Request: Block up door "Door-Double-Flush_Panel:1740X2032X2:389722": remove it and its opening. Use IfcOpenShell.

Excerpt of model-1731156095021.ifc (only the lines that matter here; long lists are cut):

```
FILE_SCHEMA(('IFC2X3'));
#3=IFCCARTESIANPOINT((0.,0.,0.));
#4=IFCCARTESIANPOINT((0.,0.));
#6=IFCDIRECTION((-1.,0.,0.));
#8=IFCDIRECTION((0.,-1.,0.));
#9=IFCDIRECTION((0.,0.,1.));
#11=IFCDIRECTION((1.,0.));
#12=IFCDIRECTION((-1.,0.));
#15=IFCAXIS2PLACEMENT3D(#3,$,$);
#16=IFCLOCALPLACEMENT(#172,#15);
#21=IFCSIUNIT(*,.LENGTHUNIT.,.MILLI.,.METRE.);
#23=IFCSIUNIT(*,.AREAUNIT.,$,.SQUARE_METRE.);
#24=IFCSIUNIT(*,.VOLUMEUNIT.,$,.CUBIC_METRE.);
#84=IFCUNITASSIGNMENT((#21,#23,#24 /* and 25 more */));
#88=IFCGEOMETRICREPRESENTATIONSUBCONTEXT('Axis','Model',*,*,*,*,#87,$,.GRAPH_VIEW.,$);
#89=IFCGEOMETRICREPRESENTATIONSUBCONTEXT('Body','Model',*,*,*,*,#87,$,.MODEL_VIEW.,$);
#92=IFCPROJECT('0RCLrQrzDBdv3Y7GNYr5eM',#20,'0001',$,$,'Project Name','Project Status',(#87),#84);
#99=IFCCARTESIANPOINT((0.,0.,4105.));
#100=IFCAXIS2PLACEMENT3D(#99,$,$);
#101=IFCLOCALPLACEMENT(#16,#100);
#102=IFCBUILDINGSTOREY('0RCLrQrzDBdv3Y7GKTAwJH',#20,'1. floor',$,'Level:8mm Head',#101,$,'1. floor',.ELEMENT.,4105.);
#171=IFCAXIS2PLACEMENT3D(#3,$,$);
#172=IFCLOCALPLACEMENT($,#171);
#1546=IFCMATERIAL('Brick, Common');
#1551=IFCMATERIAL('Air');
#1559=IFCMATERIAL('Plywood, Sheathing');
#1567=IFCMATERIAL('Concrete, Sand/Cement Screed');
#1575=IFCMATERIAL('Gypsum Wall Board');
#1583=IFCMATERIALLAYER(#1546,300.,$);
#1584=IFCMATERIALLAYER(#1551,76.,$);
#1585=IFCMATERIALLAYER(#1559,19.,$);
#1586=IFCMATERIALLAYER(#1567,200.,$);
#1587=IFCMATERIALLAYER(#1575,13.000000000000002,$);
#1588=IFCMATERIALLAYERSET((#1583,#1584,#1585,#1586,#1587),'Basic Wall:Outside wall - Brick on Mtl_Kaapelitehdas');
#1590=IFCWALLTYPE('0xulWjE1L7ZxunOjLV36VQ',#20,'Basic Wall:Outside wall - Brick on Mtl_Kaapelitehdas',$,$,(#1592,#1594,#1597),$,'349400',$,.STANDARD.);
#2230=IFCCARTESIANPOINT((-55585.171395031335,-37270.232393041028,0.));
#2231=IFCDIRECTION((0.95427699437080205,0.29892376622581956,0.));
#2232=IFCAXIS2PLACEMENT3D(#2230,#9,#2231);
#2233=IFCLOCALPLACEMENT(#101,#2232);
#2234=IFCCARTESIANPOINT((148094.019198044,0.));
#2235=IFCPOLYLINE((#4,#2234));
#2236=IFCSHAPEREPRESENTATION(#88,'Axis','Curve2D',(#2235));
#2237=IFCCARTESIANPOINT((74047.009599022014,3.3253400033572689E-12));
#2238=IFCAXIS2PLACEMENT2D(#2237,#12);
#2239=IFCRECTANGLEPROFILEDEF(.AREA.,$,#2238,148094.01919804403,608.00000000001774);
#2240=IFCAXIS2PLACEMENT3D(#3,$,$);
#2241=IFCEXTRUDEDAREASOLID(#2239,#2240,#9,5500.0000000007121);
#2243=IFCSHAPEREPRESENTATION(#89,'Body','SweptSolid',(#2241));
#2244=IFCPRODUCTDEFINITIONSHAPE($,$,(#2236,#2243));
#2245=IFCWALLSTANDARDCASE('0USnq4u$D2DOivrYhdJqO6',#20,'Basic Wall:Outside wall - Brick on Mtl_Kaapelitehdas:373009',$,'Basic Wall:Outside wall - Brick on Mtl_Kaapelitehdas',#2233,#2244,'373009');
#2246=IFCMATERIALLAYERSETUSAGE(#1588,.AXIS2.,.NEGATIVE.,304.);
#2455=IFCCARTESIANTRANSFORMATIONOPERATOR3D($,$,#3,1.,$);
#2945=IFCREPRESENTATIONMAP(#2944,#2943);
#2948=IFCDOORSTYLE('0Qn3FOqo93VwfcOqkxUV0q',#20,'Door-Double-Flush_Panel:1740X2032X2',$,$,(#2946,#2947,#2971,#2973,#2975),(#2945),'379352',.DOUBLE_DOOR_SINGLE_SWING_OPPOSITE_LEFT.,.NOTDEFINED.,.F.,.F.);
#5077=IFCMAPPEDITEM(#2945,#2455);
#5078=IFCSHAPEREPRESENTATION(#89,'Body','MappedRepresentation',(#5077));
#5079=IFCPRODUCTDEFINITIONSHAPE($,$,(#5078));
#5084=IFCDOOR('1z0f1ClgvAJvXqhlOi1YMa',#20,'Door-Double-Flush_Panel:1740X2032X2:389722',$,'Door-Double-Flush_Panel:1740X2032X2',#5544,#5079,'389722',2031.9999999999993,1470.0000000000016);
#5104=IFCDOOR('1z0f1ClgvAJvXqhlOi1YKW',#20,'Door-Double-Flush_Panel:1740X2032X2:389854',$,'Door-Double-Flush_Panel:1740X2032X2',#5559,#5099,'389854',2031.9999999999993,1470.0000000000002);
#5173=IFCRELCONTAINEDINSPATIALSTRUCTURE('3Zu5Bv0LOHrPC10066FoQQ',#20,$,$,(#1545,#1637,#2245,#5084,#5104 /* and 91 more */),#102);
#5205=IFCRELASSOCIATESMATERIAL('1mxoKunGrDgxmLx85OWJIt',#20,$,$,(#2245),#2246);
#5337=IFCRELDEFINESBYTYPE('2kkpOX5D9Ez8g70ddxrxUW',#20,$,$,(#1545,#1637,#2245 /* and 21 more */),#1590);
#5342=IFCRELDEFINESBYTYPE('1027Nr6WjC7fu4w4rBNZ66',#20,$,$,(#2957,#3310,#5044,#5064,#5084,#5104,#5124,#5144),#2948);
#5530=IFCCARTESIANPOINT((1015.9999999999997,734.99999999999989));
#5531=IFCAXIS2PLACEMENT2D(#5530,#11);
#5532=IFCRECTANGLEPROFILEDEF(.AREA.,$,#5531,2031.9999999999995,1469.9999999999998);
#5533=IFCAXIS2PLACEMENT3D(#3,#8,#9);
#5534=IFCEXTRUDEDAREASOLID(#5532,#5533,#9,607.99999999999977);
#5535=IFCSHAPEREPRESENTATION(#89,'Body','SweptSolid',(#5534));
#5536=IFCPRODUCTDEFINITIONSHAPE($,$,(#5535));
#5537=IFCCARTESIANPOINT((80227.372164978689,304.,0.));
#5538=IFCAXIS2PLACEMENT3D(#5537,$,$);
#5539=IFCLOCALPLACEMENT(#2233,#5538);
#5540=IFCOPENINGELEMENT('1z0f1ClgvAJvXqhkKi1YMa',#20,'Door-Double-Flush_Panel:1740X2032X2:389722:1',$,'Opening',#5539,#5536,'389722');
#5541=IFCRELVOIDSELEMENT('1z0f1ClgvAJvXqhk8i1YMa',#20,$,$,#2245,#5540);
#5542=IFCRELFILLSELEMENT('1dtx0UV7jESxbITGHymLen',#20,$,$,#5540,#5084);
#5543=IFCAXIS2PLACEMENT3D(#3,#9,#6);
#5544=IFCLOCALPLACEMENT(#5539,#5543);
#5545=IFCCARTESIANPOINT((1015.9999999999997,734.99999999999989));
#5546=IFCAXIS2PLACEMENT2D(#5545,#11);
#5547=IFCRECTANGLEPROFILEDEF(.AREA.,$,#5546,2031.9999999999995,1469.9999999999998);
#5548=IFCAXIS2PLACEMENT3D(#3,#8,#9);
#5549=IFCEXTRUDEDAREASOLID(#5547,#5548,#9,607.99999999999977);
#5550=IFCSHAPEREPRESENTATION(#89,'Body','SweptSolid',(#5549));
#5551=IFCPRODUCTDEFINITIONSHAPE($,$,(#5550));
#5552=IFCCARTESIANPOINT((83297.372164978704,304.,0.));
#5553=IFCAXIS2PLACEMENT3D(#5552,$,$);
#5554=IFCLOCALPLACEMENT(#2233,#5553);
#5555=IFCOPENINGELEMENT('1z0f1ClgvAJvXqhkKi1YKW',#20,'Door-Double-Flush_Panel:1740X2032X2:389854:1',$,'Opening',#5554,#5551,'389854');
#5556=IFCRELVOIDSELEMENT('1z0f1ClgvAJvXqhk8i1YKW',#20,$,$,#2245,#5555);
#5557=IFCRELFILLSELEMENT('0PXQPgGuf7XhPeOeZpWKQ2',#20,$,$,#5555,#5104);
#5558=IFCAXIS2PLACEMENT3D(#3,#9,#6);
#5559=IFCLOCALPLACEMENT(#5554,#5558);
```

```python
import ifcopenshell
import ifcopenshell.api.feature
import ifcopenshell.api.root
import ifcopenshell.geom
import ifcopenshell.util.shape

model = ifcopenshell.open("model-1731156095021.ifc")
settings = ifcopenshell.geom.settings()


def volume(element):
    """Net volume in cubic metres, openings subtracted."""
    shape = ifcopenshell.geom.create_shape(settings, element)
    return ifcopenshell.util.shape.get_volume(shape.geometry)


door = model.by_guid("1z0f1ClgvAJvXqhlOi1YMa")
opening = door.FillsVoids[0].RelatingOpeningElement
wall = opening.VoidsElements[0].RelatingBuildingElement
before = volume(wall)

ifcopenshell.api.root.remove_product(model, product=door)
ifcopenshell.api.feature.remove_feature(model, feature=opening)

after = volume(wall)

print(f"wall volume {before:.3f} -> {after:.3f} m3")

model.write("model-1731156095021_updated.ifc")
```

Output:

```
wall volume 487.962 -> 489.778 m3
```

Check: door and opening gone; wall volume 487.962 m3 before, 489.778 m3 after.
